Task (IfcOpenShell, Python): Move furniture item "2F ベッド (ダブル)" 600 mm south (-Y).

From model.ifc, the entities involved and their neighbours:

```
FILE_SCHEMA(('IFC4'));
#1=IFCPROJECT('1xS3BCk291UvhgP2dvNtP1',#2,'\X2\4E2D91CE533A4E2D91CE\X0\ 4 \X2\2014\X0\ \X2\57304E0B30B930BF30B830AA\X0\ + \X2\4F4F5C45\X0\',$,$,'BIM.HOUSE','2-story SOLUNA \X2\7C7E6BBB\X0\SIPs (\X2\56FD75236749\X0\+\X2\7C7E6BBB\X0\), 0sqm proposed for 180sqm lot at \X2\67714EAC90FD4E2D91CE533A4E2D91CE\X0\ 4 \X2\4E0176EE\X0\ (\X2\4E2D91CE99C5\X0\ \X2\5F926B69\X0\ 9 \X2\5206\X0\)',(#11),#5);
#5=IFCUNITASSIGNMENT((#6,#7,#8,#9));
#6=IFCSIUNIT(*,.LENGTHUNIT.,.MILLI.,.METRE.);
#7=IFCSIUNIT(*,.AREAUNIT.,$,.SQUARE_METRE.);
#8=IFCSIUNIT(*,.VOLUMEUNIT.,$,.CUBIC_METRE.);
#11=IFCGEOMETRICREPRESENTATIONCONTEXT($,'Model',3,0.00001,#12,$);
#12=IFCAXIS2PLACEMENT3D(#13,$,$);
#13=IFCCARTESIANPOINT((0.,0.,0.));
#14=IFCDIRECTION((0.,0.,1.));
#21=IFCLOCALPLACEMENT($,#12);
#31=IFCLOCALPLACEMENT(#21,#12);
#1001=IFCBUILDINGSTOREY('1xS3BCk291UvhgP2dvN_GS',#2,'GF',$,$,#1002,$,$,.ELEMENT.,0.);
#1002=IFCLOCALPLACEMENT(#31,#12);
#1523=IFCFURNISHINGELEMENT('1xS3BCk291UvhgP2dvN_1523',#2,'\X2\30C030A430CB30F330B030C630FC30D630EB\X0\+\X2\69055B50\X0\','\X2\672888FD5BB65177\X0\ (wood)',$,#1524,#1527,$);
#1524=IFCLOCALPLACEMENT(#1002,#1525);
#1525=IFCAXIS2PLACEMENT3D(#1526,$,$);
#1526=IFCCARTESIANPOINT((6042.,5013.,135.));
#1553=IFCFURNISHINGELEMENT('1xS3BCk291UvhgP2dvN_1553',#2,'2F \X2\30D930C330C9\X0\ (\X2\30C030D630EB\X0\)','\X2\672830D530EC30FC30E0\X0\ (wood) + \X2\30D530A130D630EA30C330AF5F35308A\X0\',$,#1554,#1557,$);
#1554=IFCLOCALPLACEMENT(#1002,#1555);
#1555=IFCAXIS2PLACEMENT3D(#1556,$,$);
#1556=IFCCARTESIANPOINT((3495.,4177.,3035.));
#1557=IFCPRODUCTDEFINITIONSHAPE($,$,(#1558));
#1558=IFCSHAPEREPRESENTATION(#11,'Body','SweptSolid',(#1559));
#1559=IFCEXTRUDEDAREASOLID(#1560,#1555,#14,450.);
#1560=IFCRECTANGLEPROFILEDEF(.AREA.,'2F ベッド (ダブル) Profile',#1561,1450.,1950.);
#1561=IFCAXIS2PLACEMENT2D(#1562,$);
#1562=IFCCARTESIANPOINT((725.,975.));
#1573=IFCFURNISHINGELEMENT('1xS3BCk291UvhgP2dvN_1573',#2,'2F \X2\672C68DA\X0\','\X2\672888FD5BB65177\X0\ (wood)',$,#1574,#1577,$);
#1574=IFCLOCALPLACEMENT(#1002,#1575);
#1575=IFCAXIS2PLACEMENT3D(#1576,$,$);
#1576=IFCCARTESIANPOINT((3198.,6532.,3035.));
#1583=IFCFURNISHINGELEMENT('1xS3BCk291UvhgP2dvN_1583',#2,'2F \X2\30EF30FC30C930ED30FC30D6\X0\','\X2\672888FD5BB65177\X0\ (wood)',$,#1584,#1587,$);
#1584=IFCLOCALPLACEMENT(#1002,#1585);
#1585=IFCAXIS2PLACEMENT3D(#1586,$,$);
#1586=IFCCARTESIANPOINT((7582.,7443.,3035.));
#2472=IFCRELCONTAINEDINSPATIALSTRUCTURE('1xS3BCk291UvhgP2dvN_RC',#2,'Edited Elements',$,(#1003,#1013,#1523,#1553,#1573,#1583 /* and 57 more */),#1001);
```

```python
import ifcopenshell
import ifcopenshell.api.geometry
import ifcopenshell.util.placement

model = ifcopenshell.open("model.ifc")

item = model.by_id(1553)
matrix = ifcopenshell.util.placement.get_local_placement(item.ObjectPlacement)
matrix[1, 3] -= 600.0
ifcopenshell.api.geometry.edit_object_placement(model, product=item, matrix=matrix, is_si=False)

print(ifcopenshell.util.placement.get_local_placement(item.ObjectPlacement).round(3) + 0.0)

model.write("model_rev.ifc")
```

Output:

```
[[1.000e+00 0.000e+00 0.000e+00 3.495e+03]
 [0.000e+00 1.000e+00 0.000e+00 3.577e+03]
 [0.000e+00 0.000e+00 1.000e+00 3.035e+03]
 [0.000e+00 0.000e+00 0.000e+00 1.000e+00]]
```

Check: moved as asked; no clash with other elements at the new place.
